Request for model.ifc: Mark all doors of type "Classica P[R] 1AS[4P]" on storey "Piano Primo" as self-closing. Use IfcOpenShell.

First a look at what the model holds.

```python
import ifcopenshell
import ifcopenshell.util.element

model = ifcopenshell.open("model.ifc")
print(model.schema)
storey = next(s for s in model.by_type("IfcBuildingStorey") if s.Name == "Piano Primo")
doors = [e for e in ifcopenshell.util.element.get_decomposition(storey) if e.is_a("IfcDoor")]
seen = {}
for e in doors:
    element_type = ifcopenshell.util.element.get_type(e)
    key = (element_type.Name if element_type != e and element_type else None, ifcopenshell.util.element.get_pset(e, "Pset_DoorCommon", "SelfClosing"))
    seen[key] = seen.get(key, 0) + 1
for (name, value), count in sorted(seen.items(), key=str):
    print(count, "x", name, "|", value)
```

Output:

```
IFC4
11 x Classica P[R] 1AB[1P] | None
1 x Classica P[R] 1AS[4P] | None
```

```python
import ifcopenshell
import ifcopenshell.api.pset
import ifcopenshell.util.element

model = ifcopenshell.open("model.ifc")

storey = next(s for s in model.by_type("IfcBuildingStorey") if s.Name == "Piano Primo")
doors = [e for e in ifcopenshell.util.element.get_decomposition(storey) if e.is_a("IfcDoor")]

count = 0
for e in doors:
    element_type = ifcopenshell.util.element.get_type(e)
    if element_type in (None, e) or element_type.Name != "Classica P[R] 1AS[4P]":
        continue
    # add_pset returns the element's existing set when there is one.
    pset = ifcopenshell.api.pset.add_pset(model, product=e, name="Pset_DoorCommon")
    ifcopenshell.api.pset.edit_pset(model, pset=pset, properties={"SelfClosing": True})
    count += 1

print(count, "doors updated")

model.write("model_edited.ifc")
```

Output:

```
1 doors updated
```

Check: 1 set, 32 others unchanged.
